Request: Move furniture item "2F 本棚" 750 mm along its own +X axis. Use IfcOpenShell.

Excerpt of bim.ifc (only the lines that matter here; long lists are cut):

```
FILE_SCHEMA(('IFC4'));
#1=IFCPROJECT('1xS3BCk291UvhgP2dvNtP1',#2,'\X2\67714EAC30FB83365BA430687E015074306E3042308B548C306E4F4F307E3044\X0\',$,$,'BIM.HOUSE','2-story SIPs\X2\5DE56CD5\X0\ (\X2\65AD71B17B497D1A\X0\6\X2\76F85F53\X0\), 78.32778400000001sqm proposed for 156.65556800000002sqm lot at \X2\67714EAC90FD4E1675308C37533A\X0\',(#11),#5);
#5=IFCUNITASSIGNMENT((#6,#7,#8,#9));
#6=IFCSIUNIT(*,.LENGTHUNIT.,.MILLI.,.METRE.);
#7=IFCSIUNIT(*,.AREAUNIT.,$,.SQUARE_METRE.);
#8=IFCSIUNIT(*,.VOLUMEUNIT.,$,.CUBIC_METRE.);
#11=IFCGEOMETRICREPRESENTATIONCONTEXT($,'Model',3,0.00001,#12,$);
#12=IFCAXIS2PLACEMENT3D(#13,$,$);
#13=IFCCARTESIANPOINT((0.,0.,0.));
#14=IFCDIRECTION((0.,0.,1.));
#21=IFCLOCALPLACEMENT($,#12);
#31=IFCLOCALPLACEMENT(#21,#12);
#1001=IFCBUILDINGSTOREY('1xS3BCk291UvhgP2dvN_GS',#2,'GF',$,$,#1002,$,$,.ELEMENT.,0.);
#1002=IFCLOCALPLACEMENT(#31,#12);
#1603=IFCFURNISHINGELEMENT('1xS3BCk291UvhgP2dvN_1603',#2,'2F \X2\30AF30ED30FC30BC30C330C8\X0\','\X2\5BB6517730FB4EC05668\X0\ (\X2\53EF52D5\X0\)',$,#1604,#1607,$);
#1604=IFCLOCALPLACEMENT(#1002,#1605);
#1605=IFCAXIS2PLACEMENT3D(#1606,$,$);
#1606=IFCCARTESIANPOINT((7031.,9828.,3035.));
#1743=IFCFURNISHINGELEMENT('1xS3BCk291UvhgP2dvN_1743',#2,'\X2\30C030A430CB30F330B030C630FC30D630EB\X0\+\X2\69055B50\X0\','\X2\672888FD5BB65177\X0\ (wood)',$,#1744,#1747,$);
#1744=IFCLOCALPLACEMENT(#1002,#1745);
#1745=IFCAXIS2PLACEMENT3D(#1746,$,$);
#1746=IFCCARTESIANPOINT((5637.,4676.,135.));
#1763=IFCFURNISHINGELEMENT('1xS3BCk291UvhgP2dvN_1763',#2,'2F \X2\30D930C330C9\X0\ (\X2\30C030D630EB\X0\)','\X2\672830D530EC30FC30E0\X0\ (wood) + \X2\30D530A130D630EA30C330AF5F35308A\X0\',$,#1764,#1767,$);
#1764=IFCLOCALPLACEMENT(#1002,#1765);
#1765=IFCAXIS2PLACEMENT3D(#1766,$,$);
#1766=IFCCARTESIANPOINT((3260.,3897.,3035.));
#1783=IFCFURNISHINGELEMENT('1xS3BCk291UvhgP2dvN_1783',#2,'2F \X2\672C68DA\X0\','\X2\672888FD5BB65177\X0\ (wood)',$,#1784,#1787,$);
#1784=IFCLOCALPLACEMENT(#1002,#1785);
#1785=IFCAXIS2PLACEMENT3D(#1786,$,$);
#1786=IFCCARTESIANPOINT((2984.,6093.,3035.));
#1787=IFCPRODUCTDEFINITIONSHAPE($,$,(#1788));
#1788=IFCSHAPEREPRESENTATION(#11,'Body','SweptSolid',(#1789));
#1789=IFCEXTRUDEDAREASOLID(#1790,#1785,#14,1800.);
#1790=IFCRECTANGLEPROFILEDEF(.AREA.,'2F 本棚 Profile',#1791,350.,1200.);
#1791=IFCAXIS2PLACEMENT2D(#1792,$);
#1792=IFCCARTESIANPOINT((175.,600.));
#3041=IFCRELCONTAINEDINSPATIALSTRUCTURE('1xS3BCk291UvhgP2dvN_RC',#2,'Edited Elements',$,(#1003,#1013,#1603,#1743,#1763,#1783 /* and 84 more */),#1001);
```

```python
import ifcopenshell
import ifcopenshell.api.geometry
import ifcopenshell.util.placement

model = ifcopenshell.open("bim.ifc")

item = model.by_guid("1xS3BCk291UvhgP2dvN_1783")
matrix = ifcopenshell.util.placement.get_local_placement(item.ObjectPlacement)
matrix[:3, 3] += matrix[:3, 0] * 750.0
ifcopenshell.api.geometry.edit_object_placement(model, product=item, matrix=matrix, is_si=False)

print(ifcopenshell.util.placement.get_local_placement(item.ObjectPlacement).round(3) + 0.0)

model.write("bim_rev.ifc")
```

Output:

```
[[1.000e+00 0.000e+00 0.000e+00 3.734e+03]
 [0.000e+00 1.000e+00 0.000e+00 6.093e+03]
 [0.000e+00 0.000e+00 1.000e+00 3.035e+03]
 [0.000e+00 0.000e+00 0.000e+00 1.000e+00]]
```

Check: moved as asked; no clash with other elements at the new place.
